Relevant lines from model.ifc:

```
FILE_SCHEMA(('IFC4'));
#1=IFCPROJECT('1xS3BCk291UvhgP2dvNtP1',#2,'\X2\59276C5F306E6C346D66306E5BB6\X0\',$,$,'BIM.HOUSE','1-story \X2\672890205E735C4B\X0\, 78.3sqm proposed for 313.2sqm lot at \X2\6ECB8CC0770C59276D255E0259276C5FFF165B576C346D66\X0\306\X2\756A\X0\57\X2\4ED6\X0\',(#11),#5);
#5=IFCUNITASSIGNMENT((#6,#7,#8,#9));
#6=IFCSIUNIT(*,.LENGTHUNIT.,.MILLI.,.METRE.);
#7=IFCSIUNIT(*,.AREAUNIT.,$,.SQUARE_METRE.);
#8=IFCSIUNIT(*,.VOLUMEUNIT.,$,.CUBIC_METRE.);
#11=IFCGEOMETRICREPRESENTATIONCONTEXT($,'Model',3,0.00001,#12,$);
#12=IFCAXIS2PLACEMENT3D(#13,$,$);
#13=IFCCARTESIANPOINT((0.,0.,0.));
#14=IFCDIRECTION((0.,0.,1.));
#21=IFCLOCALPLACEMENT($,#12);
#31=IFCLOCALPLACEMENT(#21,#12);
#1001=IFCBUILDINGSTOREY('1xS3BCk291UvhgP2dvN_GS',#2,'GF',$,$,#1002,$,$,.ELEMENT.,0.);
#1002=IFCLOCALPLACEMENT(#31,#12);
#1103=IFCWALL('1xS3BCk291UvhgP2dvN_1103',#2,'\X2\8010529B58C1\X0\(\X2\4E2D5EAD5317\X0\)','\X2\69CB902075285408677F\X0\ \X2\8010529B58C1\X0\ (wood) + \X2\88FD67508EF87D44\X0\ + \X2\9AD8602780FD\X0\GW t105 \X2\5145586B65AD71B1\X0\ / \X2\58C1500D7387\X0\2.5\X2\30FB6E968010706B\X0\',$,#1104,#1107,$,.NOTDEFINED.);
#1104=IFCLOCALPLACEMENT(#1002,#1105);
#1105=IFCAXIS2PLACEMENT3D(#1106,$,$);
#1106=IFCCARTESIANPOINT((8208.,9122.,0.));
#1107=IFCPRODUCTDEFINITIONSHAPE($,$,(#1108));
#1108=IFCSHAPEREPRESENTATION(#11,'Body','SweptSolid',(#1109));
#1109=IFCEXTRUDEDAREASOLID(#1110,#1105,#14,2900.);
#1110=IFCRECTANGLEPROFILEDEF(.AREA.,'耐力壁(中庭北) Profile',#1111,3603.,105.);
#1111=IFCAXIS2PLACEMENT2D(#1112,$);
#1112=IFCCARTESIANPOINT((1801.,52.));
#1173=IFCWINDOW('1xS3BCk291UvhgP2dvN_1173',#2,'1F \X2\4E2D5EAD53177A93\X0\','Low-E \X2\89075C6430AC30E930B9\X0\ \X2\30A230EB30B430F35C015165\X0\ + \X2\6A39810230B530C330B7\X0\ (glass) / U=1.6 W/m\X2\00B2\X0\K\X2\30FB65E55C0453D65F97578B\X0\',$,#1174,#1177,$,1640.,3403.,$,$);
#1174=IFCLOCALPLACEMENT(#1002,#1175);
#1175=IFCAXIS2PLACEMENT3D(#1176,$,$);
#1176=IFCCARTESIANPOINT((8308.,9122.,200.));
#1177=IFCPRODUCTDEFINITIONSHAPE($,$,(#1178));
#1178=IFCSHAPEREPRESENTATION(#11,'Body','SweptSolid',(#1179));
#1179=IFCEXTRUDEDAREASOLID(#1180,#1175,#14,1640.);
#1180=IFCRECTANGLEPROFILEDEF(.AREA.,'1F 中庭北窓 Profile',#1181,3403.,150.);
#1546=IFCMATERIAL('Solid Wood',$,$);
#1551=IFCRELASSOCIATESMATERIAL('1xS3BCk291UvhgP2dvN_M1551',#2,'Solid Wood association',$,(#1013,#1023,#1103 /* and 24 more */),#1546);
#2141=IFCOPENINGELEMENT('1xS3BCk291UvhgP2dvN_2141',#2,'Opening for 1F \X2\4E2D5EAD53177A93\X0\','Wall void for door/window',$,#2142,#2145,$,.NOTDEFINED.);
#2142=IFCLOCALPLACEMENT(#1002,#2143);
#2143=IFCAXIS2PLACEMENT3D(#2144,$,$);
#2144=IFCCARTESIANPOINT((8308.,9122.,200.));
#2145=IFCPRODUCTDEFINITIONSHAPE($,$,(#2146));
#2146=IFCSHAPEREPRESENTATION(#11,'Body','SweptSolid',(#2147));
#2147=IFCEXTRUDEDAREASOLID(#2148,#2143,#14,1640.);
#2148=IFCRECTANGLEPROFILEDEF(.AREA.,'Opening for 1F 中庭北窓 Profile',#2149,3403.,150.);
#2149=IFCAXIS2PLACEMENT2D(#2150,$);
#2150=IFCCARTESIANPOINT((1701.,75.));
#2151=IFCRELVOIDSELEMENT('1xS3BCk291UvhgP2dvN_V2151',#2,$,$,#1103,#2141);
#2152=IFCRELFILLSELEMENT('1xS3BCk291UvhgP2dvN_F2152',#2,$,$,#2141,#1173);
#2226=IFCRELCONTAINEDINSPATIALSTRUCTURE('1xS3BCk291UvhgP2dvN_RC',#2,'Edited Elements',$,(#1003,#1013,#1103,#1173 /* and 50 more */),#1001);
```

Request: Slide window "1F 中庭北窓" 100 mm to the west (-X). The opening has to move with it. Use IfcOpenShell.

```python
import ifcopenshell
import ifcopenshell.api.geometry
import ifcopenshell.util.placement
import ifcopenshell.util.unit

model = ifcopenshell.open("model.ifc")
unit_scale = ifcopenshell.util.unit.calculate_unit_scale(model)

window = model.by_guid("1xS3BCk291UvhgP2dvN_1173")
opening = window.FillsVoids[0].RelatingOpeningElement
wall = opening.VoidsElements[0].RelatingBuildingElement

wall_matrix = ifcopenshell.util.placement.get_local_placement(wall.ObjectPlacement)
shift = wall_matrix[:3, 0] * -0.1 / unit_scale
before = ifcopenshell.util.placement.get_local_placement(window.ObjectPlacement)[:3, 3].copy()

# The window is not placed relative to its opening, so move both.
for product in (opening, window):
    matrix = ifcopenshell.util.placement.get_local_placement(product.ObjectPlacement)
    matrix[:3, 3] += shift
    ifcopenshell.api.geometry.edit_object_placement(model, product=product, matrix=matrix, is_si=False)

after = ifcopenshell.util.placement.get_local_placement(window.ObjectPlacement)[:3, 3]
print("window moved by", (after - before).round(3) + 0.0)

model.write("model-out.ifc")
```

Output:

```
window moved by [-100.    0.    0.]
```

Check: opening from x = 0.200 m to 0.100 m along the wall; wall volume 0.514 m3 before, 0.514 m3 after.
